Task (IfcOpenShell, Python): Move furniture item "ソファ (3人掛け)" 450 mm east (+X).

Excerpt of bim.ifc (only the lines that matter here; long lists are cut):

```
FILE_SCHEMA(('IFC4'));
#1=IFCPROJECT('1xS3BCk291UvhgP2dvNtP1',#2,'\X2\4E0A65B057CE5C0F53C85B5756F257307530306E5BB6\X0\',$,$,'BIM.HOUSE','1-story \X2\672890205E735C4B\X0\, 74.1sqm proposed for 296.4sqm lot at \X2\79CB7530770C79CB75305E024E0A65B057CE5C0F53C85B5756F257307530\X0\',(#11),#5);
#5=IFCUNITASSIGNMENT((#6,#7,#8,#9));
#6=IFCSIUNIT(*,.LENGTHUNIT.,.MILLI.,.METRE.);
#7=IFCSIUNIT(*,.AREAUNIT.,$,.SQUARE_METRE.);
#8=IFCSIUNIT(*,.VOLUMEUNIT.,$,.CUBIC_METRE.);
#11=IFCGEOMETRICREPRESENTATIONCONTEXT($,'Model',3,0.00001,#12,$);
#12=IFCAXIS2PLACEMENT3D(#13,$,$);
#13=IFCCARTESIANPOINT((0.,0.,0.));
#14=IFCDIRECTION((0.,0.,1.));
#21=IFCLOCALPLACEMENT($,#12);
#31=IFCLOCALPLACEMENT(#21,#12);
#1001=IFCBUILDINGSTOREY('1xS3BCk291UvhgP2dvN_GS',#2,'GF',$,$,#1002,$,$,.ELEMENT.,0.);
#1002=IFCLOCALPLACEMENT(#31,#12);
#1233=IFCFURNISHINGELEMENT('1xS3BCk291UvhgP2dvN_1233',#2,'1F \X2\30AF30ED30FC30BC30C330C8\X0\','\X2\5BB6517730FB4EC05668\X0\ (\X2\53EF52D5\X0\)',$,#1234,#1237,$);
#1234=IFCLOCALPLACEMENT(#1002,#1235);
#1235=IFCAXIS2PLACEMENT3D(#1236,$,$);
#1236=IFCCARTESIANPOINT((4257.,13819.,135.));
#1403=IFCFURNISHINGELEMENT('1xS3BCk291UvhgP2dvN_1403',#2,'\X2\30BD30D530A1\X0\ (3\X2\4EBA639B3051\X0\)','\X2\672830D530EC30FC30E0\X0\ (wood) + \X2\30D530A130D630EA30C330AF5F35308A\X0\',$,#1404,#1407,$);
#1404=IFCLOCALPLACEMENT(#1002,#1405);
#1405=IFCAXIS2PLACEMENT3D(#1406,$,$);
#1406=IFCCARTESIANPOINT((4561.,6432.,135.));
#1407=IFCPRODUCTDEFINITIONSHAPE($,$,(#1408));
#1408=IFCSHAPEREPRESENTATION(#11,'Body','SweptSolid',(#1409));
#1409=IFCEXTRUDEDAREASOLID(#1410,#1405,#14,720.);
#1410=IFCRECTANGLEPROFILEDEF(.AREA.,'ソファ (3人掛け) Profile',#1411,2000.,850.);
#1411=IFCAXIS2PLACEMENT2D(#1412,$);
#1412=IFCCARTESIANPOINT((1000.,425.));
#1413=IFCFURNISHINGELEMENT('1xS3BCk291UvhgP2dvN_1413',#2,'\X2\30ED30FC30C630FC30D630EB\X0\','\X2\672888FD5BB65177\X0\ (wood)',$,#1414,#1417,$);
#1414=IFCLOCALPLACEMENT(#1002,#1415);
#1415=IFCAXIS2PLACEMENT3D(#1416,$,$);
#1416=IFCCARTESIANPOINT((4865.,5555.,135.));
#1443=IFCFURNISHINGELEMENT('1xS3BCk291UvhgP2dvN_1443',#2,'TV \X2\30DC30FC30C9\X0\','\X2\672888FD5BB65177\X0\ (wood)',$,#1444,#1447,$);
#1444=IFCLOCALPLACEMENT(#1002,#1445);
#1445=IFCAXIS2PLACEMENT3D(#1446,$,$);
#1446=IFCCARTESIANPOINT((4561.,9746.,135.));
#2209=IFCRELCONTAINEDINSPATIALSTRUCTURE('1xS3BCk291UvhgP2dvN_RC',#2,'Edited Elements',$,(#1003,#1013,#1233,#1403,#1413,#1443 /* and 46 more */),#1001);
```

```python
import ifcopenshell
import ifcopenshell.api.geometry
import ifcopenshell.util.placement

model = ifcopenshell.open("bim.ifc")

item = model.by_id(1403)
matrix = ifcopenshell.util.placement.get_local_placement(item.ObjectPlacement)
matrix[0, 3] += 450.0
ifcopenshell.api.geometry.edit_object_placement(model, product=item, matrix=matrix, is_si=False)

print(ifcopenshell.util.placement.get_local_placement(item.ObjectPlacement).round(3) + 0.0)

model.write("bim_rev.ifc")
```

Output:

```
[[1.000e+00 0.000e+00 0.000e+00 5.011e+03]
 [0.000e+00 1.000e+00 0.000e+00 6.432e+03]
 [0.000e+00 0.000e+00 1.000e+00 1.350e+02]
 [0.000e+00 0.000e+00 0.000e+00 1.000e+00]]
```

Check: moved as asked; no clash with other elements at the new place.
